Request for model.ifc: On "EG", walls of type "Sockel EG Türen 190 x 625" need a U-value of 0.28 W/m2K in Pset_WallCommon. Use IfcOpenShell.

First a look at what the model holds.

```python
import ifcopenshell
import ifcopenshell.util.element

model = ifcopenshell.open("model.ifc")
print(model.schema)
storey = next(s for s in model.by_type("IfcBuildingStorey") if s.Name == "EG")
walls = [e for e in ifcopenshell.util.element.get_decomposition(storey) if e.is_a("IfcWall")]
seen = {}
for e in walls:
    element_type = ifcopenshell.util.element.get_type(e)
    key = (element_type.Name if element_type != e and element_type else None, ifcopenshell.util.element.get_pset(e, "Pset_WallCommon", "ThermalTransmittance"))
    seen[key] = seen.get(key, 0) + 1
for (name, value), count in sorted(seen.items(), key=str):
    print(count, "x", name, "|", value)
```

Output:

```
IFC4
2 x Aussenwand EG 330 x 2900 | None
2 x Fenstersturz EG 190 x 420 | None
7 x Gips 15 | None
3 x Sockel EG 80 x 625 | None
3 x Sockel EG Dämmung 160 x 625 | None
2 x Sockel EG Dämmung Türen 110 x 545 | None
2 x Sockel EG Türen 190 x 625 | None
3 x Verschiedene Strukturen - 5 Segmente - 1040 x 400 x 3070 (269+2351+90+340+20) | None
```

```python
import ifcopenshell
import ifcopenshell.api.pset
import ifcopenshell.util.element

model = ifcopenshell.open("model.ifc")

storey = next(s for s in model.by_type("IfcBuildingStorey") if s.Name == "EG")
walls = [e for e in ifcopenshell.util.element.get_decomposition(storey) if e.is_a("IfcWall")]

count = 0
for e in walls:
    element_type = ifcopenshell.util.element.get_type(e)
    if element_type in (None, e) or element_type.Name != "Sockel EG Türen 190 x 625":
        continue
    # add_pset returns the element's existing set when there is one.
    pset = ifcopenshell.api.pset.add_pset(model, product=e, name="Pset_WallCommon")
    ifcopenshell.api.pset.edit_pset(model, pset=pset, properties={"ThermalTransmittance": 0.28})
    count += 1

print(count, "walls updated")

model.write("model_edited.ifc")
```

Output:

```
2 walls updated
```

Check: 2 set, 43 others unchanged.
